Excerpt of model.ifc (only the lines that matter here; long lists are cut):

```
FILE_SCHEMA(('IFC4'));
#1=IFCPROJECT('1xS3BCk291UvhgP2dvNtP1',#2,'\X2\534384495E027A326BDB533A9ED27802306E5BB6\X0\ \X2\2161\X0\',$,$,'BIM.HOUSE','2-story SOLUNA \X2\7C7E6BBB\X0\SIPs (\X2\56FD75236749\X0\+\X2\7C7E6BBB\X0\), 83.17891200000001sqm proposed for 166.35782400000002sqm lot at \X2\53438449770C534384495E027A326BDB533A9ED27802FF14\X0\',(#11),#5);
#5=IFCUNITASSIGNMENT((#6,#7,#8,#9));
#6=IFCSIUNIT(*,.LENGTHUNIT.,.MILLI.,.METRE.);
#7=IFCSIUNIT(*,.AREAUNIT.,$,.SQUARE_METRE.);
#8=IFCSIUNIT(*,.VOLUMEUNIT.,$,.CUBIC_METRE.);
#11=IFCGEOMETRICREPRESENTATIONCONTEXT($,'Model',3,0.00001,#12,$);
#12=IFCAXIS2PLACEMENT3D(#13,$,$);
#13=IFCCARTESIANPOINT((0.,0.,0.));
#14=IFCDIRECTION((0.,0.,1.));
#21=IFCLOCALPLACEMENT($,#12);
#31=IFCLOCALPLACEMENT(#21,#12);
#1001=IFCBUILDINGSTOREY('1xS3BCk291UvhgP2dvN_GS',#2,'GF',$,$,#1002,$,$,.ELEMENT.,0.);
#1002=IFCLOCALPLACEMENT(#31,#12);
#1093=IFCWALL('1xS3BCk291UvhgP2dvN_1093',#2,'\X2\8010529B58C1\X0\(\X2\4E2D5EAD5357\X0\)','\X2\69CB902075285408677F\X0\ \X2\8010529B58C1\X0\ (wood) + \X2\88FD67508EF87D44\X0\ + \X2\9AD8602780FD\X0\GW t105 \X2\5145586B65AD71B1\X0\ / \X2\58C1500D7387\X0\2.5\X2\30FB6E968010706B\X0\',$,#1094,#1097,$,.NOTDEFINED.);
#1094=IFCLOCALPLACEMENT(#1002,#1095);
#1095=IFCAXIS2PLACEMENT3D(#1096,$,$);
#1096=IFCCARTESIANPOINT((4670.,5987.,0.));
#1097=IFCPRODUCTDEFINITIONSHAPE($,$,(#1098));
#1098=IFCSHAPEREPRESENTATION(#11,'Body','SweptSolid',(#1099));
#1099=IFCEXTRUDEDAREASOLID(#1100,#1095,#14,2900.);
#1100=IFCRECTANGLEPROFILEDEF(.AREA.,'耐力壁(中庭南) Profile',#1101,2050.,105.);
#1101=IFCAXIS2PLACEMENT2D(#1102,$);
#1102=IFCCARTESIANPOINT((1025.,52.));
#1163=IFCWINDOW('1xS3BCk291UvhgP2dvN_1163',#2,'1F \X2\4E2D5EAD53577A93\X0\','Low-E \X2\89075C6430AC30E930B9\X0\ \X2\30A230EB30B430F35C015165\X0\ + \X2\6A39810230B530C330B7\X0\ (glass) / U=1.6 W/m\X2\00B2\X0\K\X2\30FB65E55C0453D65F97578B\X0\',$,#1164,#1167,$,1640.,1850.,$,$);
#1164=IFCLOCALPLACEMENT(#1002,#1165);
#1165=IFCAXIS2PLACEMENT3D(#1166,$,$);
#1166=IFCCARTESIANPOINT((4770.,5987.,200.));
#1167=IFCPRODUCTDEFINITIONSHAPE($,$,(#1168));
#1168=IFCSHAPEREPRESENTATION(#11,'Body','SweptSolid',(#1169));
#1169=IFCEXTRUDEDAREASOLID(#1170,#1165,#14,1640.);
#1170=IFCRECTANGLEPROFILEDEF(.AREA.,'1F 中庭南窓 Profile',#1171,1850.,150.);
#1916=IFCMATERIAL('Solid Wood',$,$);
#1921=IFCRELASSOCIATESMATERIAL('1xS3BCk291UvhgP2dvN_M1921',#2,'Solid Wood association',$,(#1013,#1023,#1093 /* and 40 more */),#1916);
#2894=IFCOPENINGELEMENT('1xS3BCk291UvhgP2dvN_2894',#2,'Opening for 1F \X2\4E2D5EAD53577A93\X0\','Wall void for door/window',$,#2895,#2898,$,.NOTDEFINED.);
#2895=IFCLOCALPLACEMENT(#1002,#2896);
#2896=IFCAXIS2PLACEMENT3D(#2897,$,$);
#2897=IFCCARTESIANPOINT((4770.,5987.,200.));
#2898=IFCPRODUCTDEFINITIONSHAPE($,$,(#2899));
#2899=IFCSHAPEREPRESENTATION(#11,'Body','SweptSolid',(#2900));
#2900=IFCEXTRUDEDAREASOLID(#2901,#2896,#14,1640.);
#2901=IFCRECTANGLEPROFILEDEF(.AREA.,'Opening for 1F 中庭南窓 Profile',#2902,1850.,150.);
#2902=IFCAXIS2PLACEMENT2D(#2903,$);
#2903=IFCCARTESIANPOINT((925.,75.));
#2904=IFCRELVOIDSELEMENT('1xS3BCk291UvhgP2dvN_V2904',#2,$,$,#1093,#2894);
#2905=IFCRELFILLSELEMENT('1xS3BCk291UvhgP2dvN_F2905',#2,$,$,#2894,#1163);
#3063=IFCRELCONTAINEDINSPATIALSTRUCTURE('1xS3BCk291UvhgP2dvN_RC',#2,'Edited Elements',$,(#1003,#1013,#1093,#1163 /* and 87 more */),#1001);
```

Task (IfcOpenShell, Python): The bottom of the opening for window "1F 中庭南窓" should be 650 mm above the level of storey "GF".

```python
import numpy as np
import ifcopenshell
import ifcopenshell.api.geometry
import ifcopenshell.geom
import ifcopenshell.util.element
import ifcopenshell.util.placement
import ifcopenshell.util.shape
import ifcopenshell.util.unit

model = ifcopenshell.open("model.ifc")
unit_scale = ifcopenshell.util.unit.calculate_unit_scale(model)

window = model.by_id(1163)
opening = window.FillsVoids[0].RelatingOpeningElement
storey = ifcopenshell.util.element.get_container(window, ifc_class="IfcBuildingStorey")
level = ifcopenshell.util.placement.get_local_placement(storey.ObjectPlacement)[2, 3]

# The opening's origin need not be at the sill, so measure its lowest point.
shape = ifcopenshell.geom.create_shape(ifcopenshell.geom.settings(), opening)
bottom = ifcopenshell.util.shape.get_shape_bottom_elevation(shape, shape.geometry) / unit_scale
dz = level + 650.0 - bottom

shift = np.array([0.0, 0.0, dz])
# The window is not placed relative to its opening, so move both.
for product in (opening, window):
    matrix = ifcopenshell.util.placement.get_local_placement(product.ObjectPlacement)
    matrix[:3, 3] += shift
    ifcopenshell.api.geometry.edit_object_placement(model, product=product, matrix=matrix, is_si=False)

print(f"moved by {dz * unit_scale:+.3f} m")

model.write("model_edited.ifc")
```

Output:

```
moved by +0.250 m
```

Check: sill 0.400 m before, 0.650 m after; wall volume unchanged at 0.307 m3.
